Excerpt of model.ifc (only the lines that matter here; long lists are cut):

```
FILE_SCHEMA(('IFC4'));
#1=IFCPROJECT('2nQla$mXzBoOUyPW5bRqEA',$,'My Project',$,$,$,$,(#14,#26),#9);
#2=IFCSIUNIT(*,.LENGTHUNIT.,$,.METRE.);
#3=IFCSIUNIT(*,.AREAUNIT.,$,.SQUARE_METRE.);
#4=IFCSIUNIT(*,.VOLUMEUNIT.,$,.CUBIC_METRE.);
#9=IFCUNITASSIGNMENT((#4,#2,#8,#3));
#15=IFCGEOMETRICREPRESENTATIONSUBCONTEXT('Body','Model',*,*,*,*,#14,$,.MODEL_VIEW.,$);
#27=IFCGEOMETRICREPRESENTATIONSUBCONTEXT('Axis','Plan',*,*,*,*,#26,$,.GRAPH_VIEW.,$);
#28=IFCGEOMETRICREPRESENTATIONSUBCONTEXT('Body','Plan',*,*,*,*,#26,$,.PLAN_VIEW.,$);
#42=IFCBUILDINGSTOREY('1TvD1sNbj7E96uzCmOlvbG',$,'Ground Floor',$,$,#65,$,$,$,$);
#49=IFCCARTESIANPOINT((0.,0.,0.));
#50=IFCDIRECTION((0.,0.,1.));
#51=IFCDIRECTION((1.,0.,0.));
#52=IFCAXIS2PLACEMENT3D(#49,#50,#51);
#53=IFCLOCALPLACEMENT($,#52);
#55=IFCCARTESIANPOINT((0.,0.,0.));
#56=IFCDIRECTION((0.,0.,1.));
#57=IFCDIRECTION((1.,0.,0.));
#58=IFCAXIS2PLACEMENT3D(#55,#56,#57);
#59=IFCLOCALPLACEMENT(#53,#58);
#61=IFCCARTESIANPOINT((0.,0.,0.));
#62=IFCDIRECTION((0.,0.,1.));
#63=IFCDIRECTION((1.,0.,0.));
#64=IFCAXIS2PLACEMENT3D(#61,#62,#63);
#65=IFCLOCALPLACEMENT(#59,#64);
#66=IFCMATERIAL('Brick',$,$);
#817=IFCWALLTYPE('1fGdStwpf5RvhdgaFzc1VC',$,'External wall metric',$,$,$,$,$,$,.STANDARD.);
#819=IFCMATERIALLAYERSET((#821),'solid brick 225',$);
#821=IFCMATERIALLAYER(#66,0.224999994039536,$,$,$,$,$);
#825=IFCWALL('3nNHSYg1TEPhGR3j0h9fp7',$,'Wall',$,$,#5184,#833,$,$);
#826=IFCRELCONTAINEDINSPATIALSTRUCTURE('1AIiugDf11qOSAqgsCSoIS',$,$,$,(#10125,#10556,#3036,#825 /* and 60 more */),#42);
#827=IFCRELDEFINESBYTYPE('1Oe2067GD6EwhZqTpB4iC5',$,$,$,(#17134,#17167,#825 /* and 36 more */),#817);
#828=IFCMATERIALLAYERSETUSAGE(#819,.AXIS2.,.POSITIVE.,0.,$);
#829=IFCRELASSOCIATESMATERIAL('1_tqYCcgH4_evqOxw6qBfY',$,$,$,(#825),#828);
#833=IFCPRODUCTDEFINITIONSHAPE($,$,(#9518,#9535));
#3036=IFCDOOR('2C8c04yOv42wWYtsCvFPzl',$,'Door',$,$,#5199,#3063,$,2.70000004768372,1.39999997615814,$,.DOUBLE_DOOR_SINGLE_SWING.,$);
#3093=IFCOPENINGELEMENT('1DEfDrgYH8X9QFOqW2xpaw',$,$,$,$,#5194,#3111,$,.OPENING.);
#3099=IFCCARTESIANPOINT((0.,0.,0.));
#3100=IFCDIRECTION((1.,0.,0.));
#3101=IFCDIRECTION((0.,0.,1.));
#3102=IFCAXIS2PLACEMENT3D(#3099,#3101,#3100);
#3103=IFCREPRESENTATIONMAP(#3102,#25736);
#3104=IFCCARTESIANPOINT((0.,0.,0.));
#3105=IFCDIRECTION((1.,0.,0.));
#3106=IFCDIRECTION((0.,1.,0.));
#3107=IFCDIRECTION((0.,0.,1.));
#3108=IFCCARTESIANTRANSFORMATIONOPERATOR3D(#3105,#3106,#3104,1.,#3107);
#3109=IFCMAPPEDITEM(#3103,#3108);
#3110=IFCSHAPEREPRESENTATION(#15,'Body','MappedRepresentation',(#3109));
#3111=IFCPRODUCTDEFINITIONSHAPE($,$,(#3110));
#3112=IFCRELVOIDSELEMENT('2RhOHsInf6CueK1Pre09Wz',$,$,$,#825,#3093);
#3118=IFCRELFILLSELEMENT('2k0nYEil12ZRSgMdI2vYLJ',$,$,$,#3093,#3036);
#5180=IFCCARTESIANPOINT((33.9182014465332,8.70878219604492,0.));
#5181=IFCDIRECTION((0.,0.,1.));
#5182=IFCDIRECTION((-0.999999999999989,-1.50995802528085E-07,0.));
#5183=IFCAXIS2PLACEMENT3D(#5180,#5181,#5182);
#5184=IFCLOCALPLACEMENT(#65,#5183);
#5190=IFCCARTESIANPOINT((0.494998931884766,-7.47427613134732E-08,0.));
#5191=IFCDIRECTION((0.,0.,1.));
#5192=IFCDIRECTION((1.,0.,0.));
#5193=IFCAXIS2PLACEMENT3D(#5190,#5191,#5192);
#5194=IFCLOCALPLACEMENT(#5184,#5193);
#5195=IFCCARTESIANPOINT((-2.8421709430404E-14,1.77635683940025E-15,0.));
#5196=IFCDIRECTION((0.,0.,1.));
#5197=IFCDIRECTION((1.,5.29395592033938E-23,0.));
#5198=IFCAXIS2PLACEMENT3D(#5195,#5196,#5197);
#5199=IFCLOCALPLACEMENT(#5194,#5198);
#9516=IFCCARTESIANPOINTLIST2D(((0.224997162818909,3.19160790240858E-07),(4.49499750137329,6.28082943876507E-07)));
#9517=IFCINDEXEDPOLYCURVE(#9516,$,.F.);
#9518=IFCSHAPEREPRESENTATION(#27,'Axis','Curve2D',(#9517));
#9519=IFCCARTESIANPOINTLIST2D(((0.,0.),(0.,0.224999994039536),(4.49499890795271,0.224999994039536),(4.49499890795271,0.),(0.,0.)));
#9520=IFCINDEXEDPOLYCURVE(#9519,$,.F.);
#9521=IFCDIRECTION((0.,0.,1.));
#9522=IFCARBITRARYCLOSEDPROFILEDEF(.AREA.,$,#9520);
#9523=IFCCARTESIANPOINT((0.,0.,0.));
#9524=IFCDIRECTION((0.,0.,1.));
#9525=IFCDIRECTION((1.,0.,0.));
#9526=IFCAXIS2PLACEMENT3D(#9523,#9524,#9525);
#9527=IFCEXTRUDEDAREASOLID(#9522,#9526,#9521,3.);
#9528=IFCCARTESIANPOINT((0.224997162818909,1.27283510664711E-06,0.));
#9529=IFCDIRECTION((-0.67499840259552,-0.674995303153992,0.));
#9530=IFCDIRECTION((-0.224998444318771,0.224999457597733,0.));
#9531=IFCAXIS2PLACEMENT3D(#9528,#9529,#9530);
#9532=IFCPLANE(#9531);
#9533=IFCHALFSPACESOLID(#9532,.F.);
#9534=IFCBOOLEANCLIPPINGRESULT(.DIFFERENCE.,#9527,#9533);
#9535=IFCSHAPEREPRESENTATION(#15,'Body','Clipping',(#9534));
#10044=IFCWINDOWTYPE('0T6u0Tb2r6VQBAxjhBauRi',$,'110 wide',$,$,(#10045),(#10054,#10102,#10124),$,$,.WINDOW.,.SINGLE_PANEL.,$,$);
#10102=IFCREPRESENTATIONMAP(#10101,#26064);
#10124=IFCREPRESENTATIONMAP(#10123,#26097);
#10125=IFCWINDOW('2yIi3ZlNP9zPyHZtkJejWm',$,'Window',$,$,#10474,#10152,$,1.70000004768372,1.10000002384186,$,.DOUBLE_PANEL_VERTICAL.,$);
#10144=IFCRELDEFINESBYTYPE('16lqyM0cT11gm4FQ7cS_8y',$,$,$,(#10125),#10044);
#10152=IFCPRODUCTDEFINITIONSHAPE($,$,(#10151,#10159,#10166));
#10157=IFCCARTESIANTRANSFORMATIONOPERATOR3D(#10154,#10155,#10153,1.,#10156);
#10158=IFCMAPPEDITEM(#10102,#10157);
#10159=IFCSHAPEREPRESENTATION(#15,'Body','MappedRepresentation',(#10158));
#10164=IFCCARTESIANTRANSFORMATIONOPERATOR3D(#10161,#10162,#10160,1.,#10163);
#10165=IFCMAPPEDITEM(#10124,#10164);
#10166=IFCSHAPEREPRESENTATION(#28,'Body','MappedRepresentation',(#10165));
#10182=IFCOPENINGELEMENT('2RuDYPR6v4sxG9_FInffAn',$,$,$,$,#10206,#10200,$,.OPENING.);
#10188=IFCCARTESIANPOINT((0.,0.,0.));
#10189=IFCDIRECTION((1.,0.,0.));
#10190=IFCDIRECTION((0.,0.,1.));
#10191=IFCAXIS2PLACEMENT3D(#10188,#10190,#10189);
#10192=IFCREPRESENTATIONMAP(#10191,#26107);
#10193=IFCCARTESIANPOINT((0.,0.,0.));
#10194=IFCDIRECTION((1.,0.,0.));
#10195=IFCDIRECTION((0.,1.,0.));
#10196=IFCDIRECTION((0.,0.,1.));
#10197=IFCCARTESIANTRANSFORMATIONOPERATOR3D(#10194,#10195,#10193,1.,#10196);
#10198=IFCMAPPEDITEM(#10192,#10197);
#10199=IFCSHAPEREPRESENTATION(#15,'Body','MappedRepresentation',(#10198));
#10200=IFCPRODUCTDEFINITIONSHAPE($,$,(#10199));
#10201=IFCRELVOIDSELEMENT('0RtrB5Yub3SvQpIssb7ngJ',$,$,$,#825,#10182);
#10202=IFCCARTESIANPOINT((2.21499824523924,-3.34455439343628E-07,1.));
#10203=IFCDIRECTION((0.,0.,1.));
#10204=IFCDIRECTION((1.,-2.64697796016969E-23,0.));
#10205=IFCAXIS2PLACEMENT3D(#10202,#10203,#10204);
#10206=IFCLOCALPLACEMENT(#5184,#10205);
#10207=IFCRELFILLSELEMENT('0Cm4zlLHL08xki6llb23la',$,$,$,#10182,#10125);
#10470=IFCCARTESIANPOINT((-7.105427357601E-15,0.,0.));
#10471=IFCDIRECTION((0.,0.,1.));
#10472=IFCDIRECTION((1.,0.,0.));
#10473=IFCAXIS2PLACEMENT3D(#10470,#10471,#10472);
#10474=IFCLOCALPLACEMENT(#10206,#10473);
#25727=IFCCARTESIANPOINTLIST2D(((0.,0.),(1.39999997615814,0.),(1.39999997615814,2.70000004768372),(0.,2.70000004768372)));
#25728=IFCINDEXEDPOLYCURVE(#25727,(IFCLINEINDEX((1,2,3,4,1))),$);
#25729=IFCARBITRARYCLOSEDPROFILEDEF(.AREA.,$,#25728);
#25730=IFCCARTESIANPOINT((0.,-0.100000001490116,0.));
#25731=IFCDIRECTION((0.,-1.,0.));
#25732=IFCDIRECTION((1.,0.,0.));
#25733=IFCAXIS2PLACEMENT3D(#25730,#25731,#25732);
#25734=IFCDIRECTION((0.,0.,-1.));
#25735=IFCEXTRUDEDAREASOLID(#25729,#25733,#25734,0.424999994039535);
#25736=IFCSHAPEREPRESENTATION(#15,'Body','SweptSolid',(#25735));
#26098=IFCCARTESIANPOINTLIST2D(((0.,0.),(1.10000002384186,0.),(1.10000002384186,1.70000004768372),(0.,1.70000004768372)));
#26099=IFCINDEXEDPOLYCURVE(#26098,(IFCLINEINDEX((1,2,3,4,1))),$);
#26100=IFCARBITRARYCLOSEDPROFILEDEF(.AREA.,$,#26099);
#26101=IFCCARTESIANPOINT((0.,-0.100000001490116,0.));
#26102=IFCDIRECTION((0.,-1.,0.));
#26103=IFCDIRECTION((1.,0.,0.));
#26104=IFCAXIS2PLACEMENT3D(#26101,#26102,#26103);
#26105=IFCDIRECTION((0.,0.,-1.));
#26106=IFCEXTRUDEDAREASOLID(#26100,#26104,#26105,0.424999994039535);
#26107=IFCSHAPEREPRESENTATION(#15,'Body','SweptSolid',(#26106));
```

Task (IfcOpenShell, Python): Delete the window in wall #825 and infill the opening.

```python
import ifcopenshell
import ifcopenshell.api.feature
import ifcopenshell.api.root
import ifcopenshell.geom
import ifcopenshell.util.shape

model = ifcopenshell.open("model.ifc")
settings = ifcopenshell.geom.settings()


def volume(element):
    """Net volume in cubic metres, openings subtracted."""
    shape = ifcopenshell.geom.create_shape(settings, element)
    return ifcopenshell.util.shape.get_volume(shape.geometry)


window = model.by_guid("2yIi3ZlNP9zPyHZtkJejWm")
opening = window.FillsVoids[0].RelatingOpeningElement
wall = opening.VoidsElements[0].RelatingBuildingElement
before = volume(wall)

ifcopenshell.api.root.remove_product(model, product=window)
ifcopenshell.api.feature.remove_feature(model, feature=opening)

after = volume(wall)

print(f"wall volume {before:.3f} -> {after:.3f} m3")

model.write("model_rev.ifc")
```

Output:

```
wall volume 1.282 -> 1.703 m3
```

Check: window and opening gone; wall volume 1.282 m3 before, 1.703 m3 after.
